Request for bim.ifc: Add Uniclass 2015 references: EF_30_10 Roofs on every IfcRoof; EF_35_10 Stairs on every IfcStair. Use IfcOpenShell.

First a look at what the model holds.

```python
import ifcopenshell

model = ifcopenshell.open("bim.ifc")
print(model.schema)
print("classifications:", [c.Name for c in model.by_type("IfcClassification")])
for ifc_class in ("IfcDoor", "IfcRoof", "IfcStair", "IfcWall", "IfcWindow"):
    print(ifc_class, len(model.by_type(ifc_class)))
```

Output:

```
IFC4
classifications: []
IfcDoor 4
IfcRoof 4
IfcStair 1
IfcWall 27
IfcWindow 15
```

```python
import ifcopenshell
import ifcopenshell.api.classification

model = ifcopenshell.open("bim.ifc")

system = ifcopenshell.api.classification.add_classification(model, classification="Uniclass 2015")

codes = {
    "IfcRoof": ("EF_30_10", "Roofs"),
    "IfcStair": ("EF_35_10", "Stairs"),
}
for ifc_class, (code, name) in codes.items():
    products = model.by_type(ifc_class)
    ifcopenshell.api.classification.add_reference(
        model, products=products, classification=system, identification=code, name=name
    )
    print(code, len(products))

model.write("bim_edited.ifc")
```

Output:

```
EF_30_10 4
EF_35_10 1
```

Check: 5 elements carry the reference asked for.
